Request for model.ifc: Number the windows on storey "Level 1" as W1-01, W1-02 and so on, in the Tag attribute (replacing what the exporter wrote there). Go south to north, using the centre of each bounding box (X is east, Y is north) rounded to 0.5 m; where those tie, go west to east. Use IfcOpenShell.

First a look at what the model holds.

```python
import ifcopenshell
import ifcopenshell.util.element
import ifcopenshell.util.placement

model = ifcopenshell.open("model.ifc")
print(model.schema)
storey = next(s for s in model.by_type("IfcBuildingStorey") if s.Name == "Level 1")
windows = [e for e in ifcopenshell.util.element.get_decomposition(storey) if e.is_a("IfcWindow")]
for e in sorted(windows, key=lambda e: e.id()):
    origin = ifcopenshell.util.placement.get_local_placement(e.ObjectPlacement)[:3, 3]
    print(e.id(), e.Tag, e.Name, origin.round(2) + 0.0, sep=" | ")
```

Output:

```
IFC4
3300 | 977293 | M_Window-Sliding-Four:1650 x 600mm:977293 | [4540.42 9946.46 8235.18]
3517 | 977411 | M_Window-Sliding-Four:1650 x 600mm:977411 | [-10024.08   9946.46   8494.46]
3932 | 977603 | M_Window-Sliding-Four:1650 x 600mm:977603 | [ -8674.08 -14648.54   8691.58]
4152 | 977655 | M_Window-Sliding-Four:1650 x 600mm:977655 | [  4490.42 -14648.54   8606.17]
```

```python
import ifcopenshell
import ifcopenshell.geom
import ifcopenshell.util.element
import ifcopenshell.util.shape

model = ifcopenshell.open("model.ifc")
settings = ifcopenshell.geom.settings()
settings.set("use-world-coords", True)


def centre(element):
    shape = ifcopenshell.geom.create_shape(settings, element)
    return ifcopenshell.util.shape.get_bbox_centroid(shape.geometry)


storey = next(s for s in model.by_type("IfcBuildingStorey") if s.Name == "Level 1")
windows = [e for e in ifcopenshell.util.element.get_decomposition(storey) if e.is_a("IfcWindow")]

# Insertion points can sit at a corner or the storey origin, so sort by the geometry (in metres).
centres = {e: centre(e) for e in windows}
windows.sort(key=lambda e: (round(centres[e][1] / 0.5), centres[e][0]))

for i, e in enumerate(windows, start=1):
    number = f"W1-{i:02d}"
    e.Tag = number
    print(e.id(), number)

model.write("model_v2.ifc")
```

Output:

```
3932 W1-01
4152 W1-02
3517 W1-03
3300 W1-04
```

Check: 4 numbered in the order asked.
